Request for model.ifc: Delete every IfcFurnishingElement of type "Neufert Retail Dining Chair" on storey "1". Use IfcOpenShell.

First a look at what the model holds.

```python
import ifcopenshell
import ifcopenshell.util.element

model = ifcopenshell.open("model.ifc")
print(model.schema)
storey = next(s for s in model.by_type("IfcBuildingStorey") if s.Name == "1")
furniture = [e for e in ifcopenshell.util.element.get_decomposition(storey) if e.is_a("IfcFurnishingElement")]
seen = {}
for e in furniture:
    element_type = ifcopenshell.util.element.get_type(e)
    name = element_type.Name if element_type not in (None, e) else None
    seen[name] = seen.get(name, 0) + 1
for name, count in sorted(seen.items(), key=str):
    print(count, "x", name)
```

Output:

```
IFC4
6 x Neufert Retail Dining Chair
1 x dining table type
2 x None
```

```python
import ifcopenshell
import ifcopenshell.api.root
import ifcopenshell.util.element

model = ifcopenshell.open("model.ifc")

storey = next(s for s in model.by_type("IfcBuildingStorey") if s.Name == "1")
furniture = [e for e in ifcopenshell.util.element.get_decomposition(storey) if e.is_a("IfcFurnishingElement")]
targets = [e for e in furniture if (t := ifcopenshell.util.element.get_type(e)) not in (None, e) and t.Name == "Neufert Retail Dining Chair"]

for e in targets:
    ifcopenshell.api.root.remove_product(model, product=e)
print(len(targets), "removed")

model.write("model_edited.ifc")
```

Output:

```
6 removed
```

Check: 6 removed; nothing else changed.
